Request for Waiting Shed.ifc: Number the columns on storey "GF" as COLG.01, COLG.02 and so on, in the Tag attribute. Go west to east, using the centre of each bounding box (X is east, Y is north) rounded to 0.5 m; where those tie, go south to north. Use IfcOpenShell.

First a look at what the model holds.

```python
import ifcopenshell
import ifcopenshell.util.element
import ifcopenshell.util.placement

model = ifcopenshell.open("Waiting Shed.ifc")
print(model.schema)
storey = next(s for s in model.by_type("IfcBuildingStorey") if s.Name == "GF")
columns = [e for e in ifcopenshell.util.element.get_decomposition(storey) if e.is_a("IfcColumn")]
for e in sorted(columns, key=lambda e: e.id()):
    origin = ifcopenshell.util.placement.get_local_placement(e.ObjectPlacement)[:3, 3]
    print(e.id(), e.Tag, e.Name, origin.round(2) + 0.0, sep=" | ")
```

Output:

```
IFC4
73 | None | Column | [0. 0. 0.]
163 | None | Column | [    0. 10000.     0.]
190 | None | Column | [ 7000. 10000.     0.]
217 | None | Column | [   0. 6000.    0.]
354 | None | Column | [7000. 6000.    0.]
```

```python
import ifcopenshell
import ifcopenshell.geom
import ifcopenshell.util.element
import ifcopenshell.util.shape

model = ifcopenshell.open("Waiting Shed.ifc")
settings = ifcopenshell.geom.settings()
settings.set("use-world-coords", True)


def centre(element):
    shape = ifcopenshell.geom.create_shape(settings, element)
    return ifcopenshell.util.shape.get_bbox_centroid(shape.geometry)


storey = next(s for s in model.by_type("IfcBuildingStorey") if s.Name == "GF")
columns = [e for e in ifcopenshell.util.element.get_decomposition(storey) if e.is_a("IfcColumn")]

# Insertion points can sit at a corner or the storey origin, so sort by the geometry (in metres).
centres = {e: centre(e) for e in columns}
columns.sort(key=lambda e: (round(centres[e][0] / 0.5), centres[e][1]))

for i, e in enumerate(columns, start=1):
    number = f"COLG.{i:02d}"
    e.Tag = number
    print(e.id(), number)

model.write("Waiting Shed_rev.ifc")
```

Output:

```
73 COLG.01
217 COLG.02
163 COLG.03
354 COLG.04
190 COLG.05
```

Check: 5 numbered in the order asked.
